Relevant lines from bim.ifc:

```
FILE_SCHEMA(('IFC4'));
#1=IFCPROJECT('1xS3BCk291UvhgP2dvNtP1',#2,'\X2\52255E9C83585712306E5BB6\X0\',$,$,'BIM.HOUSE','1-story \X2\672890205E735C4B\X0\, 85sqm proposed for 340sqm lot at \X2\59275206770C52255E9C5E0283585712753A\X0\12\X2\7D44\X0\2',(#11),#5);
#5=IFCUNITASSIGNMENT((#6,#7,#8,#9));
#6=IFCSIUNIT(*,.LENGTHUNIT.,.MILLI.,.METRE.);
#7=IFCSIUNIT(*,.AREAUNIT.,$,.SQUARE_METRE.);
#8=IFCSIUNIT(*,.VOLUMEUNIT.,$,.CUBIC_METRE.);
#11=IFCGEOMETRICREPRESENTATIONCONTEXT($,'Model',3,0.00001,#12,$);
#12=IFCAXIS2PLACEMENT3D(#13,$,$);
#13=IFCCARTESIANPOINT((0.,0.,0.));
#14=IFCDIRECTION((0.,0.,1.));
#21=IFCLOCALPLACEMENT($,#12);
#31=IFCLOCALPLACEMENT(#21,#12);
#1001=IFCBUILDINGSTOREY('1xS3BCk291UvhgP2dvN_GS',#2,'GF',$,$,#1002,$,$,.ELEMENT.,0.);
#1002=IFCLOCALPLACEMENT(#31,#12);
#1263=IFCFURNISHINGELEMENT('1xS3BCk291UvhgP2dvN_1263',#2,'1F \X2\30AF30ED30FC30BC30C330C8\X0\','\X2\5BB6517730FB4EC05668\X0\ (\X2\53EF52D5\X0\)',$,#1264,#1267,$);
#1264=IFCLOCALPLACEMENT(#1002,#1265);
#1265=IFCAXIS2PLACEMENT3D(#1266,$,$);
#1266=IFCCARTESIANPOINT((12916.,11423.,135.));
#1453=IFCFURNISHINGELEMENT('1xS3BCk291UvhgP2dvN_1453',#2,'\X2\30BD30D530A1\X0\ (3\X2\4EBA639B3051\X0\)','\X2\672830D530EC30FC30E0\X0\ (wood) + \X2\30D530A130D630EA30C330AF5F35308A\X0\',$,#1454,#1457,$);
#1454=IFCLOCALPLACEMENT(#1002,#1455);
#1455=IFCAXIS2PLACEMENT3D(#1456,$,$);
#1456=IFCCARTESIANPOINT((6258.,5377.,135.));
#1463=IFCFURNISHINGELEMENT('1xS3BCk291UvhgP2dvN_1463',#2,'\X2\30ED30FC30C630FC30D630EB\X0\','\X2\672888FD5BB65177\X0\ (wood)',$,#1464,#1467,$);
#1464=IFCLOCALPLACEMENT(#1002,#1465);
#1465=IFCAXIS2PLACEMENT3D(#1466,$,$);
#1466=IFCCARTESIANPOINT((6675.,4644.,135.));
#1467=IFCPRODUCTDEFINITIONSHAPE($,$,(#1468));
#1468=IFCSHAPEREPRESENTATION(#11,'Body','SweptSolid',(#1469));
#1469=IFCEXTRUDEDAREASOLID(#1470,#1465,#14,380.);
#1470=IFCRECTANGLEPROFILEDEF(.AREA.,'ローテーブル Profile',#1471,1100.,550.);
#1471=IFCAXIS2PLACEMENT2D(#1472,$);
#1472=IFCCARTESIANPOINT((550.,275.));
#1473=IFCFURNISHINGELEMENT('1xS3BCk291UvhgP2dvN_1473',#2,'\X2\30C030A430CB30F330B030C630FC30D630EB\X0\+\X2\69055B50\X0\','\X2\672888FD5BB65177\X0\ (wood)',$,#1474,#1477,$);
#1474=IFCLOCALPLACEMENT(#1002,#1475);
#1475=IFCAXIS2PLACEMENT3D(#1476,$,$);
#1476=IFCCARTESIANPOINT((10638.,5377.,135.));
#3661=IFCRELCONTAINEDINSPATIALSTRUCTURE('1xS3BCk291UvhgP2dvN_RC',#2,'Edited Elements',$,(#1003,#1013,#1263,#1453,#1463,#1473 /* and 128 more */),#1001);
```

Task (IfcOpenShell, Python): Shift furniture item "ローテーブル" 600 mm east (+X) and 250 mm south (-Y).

```python
import ifcopenshell
import ifcopenshell.api.geometry
import ifcopenshell.util.placement
import ifcopenshell.util.unit

model = ifcopenshell.open("bim.ifc")
unit_scale = ifcopenshell.util.unit.calculate_unit_scale(model)

item = model.by_guid("1xS3BCk291UvhgP2dvN_1463")
matrix = ifcopenshell.util.placement.get_local_placement(item.ObjectPlacement)
matrix[0, 3] += 0.6 / unit_scale
matrix[1, 3] -= 0.25 / unit_scale
ifcopenshell.api.geometry.edit_object_placement(model, product=item, matrix=matrix, is_si=False)

print(ifcopenshell.util.placement.get_local_placement(item.ObjectPlacement).round(3) + 0.0)

model.write("bim_rev.ifc")
```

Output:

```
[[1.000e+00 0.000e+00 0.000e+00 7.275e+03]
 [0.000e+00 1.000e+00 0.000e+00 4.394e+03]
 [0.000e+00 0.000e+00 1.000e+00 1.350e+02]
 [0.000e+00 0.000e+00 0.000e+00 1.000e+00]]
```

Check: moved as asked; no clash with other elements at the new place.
